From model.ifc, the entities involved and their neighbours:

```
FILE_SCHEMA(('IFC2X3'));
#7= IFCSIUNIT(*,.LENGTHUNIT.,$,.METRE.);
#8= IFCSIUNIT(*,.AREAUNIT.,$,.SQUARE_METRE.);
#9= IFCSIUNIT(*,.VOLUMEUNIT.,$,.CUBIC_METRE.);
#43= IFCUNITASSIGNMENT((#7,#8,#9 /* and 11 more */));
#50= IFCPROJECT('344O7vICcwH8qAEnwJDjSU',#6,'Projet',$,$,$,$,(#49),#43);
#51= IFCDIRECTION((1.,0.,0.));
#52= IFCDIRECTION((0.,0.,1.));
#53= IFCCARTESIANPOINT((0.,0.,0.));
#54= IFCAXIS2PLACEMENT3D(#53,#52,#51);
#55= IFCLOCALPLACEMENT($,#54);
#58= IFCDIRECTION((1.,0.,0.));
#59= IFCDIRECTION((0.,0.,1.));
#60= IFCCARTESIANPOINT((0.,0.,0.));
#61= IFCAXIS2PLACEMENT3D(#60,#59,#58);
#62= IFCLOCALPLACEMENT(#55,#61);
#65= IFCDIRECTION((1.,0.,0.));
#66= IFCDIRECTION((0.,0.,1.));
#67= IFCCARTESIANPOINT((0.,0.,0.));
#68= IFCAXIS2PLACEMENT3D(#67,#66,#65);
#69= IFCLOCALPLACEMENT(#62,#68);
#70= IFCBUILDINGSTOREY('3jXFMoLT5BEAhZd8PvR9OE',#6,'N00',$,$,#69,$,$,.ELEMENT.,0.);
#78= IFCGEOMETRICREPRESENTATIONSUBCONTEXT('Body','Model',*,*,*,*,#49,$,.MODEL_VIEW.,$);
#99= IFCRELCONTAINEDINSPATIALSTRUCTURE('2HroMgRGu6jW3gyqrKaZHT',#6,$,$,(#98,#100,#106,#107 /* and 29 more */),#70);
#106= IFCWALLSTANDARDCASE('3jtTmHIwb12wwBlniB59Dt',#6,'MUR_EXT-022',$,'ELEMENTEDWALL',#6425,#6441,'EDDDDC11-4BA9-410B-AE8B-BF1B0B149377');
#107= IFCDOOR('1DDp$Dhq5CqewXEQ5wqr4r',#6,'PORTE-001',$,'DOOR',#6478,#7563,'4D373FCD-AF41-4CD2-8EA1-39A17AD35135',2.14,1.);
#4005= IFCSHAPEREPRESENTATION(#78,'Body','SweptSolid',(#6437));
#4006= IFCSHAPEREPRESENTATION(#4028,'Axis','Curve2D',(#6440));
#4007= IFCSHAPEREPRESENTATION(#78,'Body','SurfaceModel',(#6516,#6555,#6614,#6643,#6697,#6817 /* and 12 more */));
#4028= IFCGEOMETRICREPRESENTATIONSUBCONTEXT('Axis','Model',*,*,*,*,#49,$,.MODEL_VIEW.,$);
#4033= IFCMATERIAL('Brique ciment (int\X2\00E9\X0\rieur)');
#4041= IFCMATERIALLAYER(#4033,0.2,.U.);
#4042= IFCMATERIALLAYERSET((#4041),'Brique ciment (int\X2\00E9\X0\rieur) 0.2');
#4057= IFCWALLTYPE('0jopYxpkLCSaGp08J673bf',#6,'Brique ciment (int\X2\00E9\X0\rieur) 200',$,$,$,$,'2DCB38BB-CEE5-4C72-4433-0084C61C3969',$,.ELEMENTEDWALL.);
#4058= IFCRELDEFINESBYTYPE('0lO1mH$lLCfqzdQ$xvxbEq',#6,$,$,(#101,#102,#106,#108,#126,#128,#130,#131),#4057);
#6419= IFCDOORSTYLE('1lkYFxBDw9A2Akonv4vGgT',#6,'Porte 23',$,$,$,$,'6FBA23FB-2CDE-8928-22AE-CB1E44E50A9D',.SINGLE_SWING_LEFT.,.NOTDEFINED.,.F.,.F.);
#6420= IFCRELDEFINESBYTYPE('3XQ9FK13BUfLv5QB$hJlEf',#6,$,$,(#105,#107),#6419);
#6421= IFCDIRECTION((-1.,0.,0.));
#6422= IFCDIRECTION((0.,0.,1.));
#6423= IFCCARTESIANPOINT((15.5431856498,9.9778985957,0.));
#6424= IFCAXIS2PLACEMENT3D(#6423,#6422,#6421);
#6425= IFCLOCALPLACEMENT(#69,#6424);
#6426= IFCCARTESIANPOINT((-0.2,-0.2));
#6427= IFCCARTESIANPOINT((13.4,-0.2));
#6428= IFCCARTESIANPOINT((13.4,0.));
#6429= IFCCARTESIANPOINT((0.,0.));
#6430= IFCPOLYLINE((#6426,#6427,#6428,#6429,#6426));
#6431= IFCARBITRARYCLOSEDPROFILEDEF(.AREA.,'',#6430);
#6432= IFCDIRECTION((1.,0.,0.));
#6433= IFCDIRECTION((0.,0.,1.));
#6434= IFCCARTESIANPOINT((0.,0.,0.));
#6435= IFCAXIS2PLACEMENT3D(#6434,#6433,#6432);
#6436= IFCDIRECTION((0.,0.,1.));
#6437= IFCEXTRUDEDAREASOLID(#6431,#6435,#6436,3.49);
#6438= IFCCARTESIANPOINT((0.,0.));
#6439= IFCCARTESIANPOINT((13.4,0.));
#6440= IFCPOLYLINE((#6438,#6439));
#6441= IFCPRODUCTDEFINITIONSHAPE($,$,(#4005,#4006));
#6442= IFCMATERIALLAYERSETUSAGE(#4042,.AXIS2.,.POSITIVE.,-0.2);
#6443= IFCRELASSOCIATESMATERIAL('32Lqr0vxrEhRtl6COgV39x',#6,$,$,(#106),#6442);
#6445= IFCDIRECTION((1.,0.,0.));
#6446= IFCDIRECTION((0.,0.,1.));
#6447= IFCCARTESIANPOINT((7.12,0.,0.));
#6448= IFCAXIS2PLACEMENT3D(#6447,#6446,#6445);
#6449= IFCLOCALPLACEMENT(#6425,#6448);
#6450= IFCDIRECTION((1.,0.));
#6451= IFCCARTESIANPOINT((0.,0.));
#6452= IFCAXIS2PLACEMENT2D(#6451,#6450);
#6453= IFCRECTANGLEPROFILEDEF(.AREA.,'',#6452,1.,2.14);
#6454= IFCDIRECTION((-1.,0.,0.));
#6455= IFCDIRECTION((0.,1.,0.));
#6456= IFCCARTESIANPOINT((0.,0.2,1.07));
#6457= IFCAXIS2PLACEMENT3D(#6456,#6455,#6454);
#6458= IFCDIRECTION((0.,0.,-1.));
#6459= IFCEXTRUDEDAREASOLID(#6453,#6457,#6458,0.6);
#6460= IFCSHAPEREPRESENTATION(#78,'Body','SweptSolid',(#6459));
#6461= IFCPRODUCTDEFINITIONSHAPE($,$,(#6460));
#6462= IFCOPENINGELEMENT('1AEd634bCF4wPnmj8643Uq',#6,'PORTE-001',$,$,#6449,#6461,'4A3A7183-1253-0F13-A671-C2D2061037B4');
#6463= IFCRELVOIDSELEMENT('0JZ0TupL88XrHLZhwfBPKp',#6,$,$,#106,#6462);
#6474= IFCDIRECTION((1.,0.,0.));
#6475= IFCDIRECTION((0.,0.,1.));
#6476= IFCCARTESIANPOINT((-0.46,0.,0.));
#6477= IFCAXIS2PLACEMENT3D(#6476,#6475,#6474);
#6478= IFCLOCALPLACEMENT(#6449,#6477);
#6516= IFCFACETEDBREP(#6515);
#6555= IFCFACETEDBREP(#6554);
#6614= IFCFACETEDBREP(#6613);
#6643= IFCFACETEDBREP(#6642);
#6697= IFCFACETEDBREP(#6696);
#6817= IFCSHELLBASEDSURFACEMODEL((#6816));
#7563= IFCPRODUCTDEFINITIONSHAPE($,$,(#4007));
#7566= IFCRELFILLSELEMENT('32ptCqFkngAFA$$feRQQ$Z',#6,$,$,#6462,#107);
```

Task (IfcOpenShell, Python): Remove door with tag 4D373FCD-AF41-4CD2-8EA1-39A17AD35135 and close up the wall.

```python
import ifcopenshell
import ifcopenshell.api.feature
import ifcopenshell.api.root
import ifcopenshell.geom
import ifcopenshell.util.shape

model = ifcopenshell.open("model.ifc")
settings = ifcopenshell.geom.settings()


def volume(element):
    """Net volume in cubic metres, openings subtracted."""
    shape = ifcopenshell.geom.create_shape(settings, element)
    return ifcopenshell.util.shape.get_volume(shape.geometry)


door = model.by_guid("1DDp$Dhq5CqewXEQ5wqr4r")
opening = door.FillsVoids[0].RelatingOpeningElement
wall = opening.VoidsElements[0].RelatingBuildingElement
before = volume(wall)

ifcopenshell.api.root.remove_product(model, product=door)
ifcopenshell.api.feature.remove_feature(model, feature=opening)

after = volume(wall)

print(f"wall volume {before:.3f} -> {after:.3f} m3")

model.write("model_edited.ifc")
```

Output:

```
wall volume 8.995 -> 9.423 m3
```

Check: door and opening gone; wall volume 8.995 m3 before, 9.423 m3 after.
